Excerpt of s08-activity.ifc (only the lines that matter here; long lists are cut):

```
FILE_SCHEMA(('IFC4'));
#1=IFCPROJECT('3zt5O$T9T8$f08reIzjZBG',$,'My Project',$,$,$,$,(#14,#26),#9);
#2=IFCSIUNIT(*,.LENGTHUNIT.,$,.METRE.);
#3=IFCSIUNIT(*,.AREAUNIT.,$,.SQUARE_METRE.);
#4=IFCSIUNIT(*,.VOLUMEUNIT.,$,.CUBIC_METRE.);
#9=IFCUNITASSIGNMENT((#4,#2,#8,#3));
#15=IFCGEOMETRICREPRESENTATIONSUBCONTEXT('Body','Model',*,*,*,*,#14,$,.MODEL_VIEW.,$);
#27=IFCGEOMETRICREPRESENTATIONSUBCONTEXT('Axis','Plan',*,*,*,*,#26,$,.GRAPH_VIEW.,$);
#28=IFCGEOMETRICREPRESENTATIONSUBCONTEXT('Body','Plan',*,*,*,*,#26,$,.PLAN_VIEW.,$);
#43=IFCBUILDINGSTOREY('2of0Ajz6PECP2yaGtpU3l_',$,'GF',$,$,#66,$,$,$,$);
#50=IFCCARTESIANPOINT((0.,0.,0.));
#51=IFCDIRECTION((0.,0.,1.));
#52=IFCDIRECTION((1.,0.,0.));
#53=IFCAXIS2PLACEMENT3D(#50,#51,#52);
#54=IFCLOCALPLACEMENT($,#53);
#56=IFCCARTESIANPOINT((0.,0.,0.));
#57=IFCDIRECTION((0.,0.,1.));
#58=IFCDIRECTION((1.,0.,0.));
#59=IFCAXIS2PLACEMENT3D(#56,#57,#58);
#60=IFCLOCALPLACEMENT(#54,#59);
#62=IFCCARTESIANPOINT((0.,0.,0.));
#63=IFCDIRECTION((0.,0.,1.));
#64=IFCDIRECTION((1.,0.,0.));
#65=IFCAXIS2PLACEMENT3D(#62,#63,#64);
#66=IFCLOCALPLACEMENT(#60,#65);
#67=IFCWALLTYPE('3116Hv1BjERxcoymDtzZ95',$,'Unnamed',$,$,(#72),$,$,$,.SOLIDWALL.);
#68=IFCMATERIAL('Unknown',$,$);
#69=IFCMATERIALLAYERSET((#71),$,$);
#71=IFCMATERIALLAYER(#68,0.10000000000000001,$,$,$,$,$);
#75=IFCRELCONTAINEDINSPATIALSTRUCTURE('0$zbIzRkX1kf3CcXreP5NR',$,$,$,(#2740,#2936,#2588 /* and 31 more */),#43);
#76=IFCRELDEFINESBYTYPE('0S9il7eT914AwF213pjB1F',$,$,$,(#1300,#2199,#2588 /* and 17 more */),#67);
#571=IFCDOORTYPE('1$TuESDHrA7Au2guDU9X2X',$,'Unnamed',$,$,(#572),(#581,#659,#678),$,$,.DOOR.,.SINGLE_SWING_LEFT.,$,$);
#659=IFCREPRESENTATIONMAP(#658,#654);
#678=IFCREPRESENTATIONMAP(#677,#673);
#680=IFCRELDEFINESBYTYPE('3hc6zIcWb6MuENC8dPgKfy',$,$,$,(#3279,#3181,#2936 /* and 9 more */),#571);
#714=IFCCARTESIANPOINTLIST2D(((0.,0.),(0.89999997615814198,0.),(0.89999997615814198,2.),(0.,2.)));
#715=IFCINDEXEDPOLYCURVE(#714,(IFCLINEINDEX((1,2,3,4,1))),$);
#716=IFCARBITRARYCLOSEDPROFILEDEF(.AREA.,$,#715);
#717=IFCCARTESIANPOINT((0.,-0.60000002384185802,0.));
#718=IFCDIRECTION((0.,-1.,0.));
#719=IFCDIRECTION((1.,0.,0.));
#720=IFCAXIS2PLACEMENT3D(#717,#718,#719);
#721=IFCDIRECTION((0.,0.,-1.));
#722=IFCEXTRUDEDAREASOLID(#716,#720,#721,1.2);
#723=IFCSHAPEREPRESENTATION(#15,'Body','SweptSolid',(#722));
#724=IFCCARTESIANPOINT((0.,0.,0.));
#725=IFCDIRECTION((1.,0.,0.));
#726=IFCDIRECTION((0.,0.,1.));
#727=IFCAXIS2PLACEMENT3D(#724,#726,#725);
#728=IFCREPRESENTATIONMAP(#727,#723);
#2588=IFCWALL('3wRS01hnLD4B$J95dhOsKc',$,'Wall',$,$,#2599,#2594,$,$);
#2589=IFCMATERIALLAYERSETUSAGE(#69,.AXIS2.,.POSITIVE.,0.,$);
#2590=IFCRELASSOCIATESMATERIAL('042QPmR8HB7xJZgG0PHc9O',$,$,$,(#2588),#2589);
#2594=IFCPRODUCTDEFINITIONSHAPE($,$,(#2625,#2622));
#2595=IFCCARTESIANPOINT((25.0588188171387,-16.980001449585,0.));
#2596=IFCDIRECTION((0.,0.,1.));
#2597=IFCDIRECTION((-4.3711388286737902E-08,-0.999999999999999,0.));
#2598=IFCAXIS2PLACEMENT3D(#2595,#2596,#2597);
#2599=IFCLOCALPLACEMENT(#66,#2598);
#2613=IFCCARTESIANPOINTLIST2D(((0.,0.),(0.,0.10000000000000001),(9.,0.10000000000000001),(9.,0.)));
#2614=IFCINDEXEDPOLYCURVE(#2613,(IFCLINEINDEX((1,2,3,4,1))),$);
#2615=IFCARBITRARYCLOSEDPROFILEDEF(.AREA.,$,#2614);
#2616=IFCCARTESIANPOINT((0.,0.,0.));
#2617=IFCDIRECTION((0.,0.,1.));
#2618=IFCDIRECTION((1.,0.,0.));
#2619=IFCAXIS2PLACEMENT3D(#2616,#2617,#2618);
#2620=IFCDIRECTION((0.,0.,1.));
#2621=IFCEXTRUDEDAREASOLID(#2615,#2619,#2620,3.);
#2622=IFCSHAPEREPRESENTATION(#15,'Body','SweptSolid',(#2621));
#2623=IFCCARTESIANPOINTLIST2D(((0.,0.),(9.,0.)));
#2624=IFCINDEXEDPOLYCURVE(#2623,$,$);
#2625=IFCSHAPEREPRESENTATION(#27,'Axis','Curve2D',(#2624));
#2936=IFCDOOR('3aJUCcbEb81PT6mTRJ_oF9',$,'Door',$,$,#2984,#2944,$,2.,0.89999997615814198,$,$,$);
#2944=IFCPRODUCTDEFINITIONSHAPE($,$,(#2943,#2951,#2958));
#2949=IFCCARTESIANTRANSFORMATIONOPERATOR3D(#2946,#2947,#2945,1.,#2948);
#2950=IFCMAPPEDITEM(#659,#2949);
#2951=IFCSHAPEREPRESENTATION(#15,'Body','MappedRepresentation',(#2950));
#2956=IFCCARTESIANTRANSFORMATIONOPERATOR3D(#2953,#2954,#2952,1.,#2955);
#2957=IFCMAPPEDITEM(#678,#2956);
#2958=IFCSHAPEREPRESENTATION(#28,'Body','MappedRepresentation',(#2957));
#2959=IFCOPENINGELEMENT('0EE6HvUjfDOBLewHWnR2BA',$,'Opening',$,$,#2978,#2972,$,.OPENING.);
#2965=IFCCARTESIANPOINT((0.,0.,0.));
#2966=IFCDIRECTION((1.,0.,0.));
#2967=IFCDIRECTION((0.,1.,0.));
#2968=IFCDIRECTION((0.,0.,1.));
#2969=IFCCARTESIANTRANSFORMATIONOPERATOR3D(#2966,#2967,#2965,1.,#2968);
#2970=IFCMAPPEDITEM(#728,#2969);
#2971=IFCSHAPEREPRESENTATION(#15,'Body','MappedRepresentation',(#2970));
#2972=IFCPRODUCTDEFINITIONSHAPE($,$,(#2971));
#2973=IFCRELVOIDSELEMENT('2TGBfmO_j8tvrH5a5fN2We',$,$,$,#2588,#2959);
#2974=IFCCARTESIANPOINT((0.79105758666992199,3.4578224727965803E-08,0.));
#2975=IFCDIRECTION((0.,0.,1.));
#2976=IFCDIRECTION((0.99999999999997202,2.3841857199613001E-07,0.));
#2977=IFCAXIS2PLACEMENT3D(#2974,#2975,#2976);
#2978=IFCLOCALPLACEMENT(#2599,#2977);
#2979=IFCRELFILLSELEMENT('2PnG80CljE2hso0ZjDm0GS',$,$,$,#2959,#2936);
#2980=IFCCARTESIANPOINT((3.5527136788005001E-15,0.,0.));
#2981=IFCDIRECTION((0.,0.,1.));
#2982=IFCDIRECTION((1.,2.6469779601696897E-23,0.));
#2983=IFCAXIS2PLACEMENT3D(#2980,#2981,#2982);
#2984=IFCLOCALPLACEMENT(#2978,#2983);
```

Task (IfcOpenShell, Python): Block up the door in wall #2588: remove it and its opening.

```python
import ifcopenshell
import ifcopenshell.api.feature
import ifcopenshell.api.root
import ifcopenshell.geom
import ifcopenshell.util.shape

model = ifcopenshell.open("s08-activity.ifc")
settings = ifcopenshell.geom.settings()


def volume(element):
    """Net volume in cubic metres, openings subtracted."""
    shape = ifcopenshell.geom.create_shape(settings, element)
    return ifcopenshell.util.shape.get_volume(shape.geometry)


door = model.by_guid("3aJUCcbEb81PT6mTRJ_oF9")
opening = door.FillsVoids[0].RelatingOpeningElement
wall = opening.VoidsElements[0].RelatingBuildingElement
before = volume(wall)

ifcopenshell.api.root.remove_product(model, product=door)
ifcopenshell.api.feature.remove_feature(model, feature=opening)

after = volume(wall)

print(f"wall volume {before:.3f} -> {after:.3f} m3")

model.write("s08-activity_edited.ifc")
```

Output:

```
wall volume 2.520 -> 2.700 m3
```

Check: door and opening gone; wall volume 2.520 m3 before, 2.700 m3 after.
